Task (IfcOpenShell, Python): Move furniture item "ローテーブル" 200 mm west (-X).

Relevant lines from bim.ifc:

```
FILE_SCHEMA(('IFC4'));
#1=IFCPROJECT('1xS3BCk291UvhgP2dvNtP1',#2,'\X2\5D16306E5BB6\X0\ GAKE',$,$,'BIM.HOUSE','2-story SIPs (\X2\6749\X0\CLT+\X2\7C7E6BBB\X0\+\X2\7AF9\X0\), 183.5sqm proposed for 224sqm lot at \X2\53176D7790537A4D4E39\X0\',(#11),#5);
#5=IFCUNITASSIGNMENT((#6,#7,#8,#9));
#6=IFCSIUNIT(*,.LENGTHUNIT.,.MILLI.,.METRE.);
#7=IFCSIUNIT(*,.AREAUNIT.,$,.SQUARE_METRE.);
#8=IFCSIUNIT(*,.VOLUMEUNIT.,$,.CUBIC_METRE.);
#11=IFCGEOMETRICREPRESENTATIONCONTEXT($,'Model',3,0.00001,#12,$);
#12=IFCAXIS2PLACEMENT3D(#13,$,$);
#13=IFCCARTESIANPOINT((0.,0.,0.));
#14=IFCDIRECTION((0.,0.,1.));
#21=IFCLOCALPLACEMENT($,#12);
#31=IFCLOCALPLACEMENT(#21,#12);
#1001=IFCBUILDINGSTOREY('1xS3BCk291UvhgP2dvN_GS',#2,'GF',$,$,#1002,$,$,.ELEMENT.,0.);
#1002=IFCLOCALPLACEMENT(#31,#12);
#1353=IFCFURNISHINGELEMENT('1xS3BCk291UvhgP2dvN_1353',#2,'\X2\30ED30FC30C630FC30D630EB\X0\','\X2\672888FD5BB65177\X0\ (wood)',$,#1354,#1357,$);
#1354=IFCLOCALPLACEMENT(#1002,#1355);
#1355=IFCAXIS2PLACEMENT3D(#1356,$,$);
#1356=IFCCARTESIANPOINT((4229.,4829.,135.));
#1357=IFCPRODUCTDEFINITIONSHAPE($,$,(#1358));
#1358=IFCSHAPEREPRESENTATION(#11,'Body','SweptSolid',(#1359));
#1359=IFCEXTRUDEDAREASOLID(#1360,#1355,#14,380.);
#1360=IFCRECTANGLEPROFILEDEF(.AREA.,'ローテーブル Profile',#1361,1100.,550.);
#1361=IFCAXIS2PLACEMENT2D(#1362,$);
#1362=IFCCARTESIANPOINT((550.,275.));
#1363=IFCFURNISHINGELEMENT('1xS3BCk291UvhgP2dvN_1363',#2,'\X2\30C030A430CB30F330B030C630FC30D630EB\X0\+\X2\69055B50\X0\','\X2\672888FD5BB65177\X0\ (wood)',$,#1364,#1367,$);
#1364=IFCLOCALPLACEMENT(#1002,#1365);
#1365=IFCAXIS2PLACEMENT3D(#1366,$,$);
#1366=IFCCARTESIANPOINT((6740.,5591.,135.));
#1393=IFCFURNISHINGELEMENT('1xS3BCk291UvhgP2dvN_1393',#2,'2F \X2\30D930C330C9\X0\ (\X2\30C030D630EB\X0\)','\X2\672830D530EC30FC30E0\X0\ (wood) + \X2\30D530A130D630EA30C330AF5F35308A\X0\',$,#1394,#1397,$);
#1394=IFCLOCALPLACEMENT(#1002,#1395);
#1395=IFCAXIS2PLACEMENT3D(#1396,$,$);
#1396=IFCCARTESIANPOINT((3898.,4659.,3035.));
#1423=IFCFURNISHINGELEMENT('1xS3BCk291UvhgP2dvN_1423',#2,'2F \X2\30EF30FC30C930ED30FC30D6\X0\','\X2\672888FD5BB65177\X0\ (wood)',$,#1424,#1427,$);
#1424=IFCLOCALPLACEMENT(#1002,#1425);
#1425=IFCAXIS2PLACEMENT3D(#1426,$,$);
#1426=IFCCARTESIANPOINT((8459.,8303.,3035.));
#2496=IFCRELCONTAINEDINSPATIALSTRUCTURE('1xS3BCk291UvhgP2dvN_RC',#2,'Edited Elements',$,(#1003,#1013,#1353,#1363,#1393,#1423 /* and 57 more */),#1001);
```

```python
import ifcopenshell
import ifcopenshell.api.geometry
import ifcopenshell.util.placement
import ifcopenshell.util.unit

model = ifcopenshell.open("bim.ifc")
unit_scale = ifcopenshell.util.unit.calculate_unit_scale(model)

item = model.by_guid("1xS3BCk291UvhgP2dvN_1353")
matrix = ifcopenshell.util.placement.get_local_placement(item.ObjectPlacement)
matrix[0, 3] -= 0.2 / unit_scale
ifcopenshell.api.geometry.edit_object_placement(model, product=item, matrix=matrix, is_si=False)

print(ifcopenshell.util.placement.get_local_placement(item.ObjectPlacement).round(3) + 0.0)

model.write("bim_v2.ifc")
```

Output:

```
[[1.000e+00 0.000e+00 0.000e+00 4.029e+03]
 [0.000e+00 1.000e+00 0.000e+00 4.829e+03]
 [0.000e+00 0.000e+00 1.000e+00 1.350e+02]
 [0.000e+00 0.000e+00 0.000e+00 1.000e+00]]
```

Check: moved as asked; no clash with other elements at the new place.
